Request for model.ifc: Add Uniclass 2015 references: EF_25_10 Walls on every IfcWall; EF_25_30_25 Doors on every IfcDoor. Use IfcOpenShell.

First a look at what the model holds.

```python
import ifcopenshell

model = ifcopenshell.open("model.ifc")
print(model.schema)
print("classifications:", [c.Name for c in model.by_type("IfcClassification")])
for ifc_class in ("IfcDoor", "IfcRoof", "IfcStair", "IfcWall", "IfcWindow"):
    print(ifc_class, len(model.by_type(ifc_class)))
```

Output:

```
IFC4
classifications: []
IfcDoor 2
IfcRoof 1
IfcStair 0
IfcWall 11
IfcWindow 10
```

```python
import ifcopenshell
import ifcopenshell.api.classification

model = ifcopenshell.open("model.ifc")

system = ifcopenshell.api.classification.add_classification(model, classification="Uniclass 2015")

codes = {
    "IfcWall": ("EF_25_10", "Walls"),
    "IfcDoor": ("EF_25_30_25", "Doors"),
}
for ifc_class, (code, name) in codes.items():
    products = model.by_type(ifc_class)
    ifcopenshell.api.classification.add_reference(
        model, products=products, classification=system, identification=code, name=name
    )
    print(code, len(products))

model.write("model_edited.ifc")
```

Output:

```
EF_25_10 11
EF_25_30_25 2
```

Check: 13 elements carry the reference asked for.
